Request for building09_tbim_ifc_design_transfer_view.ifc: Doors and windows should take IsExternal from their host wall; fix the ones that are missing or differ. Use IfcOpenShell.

First a look at what the model holds.

```python
import ifcopenshell
import ifcopenshell.util.element

model = ifcopenshell.open("building09_tbim_ifc_design_transfer_view.ifc")
print(model.schema)
seen = {}
for e in model.by_type("IfcDoor") + model.by_type("IfcWindow"):
    if not e.FillsVoids:
        continue
    host = e.FillsVoids[0].RelatingOpeningElement.VoidsElements[0].RelatingBuildingElement
    own = ifcopenshell.util.element.get_pset(e, f"Pset_{e.is_a()[3:].removesuffix('StandardCase')}Common", "IsExternal")
    wall = ifcopenshell.util.element.get_pset(host, "Pset_WallCommon", "IsExternal")
    seen[e.is_a(), own, wall] = seen.get((e.is_a(), own, wall), 0) + 1
for (cls, own, wall), count in sorted(seen.items(), key=str):
    print(count, cls, "IsExternal:", own, "| host wall:", wall)
```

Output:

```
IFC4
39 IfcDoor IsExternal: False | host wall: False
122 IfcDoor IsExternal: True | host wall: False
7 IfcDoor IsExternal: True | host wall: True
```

```python
import ifcopenshell
import ifcopenshell.api.pset
import ifcopenshell.util.element

model = ifcopenshell.open("building09_tbim_ifc_design_transfer_view.ifc")

count = 0
for ifc_class, pset_name in (("IfcDoor", "Pset_DoorCommon"), ("IfcWindow", "Pset_WindowCommon")):
    for e in model.by_type(ifc_class):
        if not e.FillsVoids:
            continue
        host = e.FillsVoids[0].RelatingOpeningElement.VoidsElements[0].RelatingBuildingElement
        external = ifcopenshell.util.element.get_pset(host, "Pset_WallCommon", "IsExternal")
        if external is None or ifcopenshell.util.element.get_pset(e, pset_name, "IsExternal") == external:
            continue
        pset = ifcopenshell.api.pset.add_pset(model, product=e, name=pset_name)
        ifcopenshell.api.pset.edit_pset(model, pset=pset, properties={"IsExternal": external})
        count += 1

print(count, "updated")

model.write("building09_tbim_ifc_design_transfer_view-out.ifc")
```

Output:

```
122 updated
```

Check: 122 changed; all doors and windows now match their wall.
